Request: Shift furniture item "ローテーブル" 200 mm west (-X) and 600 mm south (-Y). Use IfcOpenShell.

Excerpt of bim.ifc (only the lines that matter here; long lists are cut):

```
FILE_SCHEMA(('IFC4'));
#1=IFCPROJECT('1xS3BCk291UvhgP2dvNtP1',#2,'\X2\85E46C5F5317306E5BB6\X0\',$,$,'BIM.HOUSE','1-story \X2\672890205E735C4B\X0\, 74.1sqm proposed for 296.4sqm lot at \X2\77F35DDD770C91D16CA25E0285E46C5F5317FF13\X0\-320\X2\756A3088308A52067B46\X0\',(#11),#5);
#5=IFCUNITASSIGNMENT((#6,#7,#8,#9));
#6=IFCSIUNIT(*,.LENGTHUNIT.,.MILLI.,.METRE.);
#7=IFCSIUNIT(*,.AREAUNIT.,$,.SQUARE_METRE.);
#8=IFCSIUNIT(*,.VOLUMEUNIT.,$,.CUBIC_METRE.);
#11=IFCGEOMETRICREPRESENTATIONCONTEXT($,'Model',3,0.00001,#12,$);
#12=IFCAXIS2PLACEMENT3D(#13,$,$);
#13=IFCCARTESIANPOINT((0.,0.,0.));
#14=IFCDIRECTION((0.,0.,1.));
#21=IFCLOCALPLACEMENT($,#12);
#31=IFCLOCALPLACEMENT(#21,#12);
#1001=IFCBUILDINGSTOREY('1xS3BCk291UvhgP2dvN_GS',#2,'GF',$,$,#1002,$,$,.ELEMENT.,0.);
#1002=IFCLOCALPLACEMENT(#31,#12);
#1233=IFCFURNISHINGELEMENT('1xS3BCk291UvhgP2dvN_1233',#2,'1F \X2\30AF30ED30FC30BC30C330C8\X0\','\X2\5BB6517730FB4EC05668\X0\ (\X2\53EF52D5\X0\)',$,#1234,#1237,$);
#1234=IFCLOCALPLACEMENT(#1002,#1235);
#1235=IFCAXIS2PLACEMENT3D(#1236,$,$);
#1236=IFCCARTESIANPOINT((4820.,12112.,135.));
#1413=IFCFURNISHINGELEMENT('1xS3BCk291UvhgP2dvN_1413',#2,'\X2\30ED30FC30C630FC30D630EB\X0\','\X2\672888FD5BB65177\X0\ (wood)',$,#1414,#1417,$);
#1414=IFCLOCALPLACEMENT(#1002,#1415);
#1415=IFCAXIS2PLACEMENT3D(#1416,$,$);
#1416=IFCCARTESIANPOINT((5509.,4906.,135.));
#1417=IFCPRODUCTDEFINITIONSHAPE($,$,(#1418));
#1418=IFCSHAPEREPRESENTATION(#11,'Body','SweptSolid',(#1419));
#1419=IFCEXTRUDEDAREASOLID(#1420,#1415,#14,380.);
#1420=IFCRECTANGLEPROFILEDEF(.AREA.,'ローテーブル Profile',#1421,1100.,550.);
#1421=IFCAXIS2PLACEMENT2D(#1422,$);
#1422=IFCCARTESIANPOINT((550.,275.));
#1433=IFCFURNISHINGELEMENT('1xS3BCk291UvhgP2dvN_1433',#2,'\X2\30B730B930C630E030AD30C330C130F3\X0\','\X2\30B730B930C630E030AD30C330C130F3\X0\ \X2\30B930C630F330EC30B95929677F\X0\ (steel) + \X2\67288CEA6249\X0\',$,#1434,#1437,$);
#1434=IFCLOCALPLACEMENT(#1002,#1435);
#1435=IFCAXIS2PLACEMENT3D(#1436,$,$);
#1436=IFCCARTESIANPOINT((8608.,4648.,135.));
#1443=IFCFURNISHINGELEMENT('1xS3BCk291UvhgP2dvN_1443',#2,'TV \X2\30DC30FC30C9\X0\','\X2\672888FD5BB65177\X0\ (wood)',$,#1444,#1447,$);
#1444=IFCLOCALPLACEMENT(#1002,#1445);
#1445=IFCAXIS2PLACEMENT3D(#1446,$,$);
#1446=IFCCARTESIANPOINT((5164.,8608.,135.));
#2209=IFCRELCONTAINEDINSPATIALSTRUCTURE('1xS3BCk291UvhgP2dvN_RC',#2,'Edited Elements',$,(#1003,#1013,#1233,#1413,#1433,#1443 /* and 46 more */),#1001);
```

```python
import ifcopenshell
import ifcopenshell.api.geometry
import ifcopenshell.util.placement
import ifcopenshell.util.unit

model = ifcopenshell.open("bim.ifc")
unit_scale = ifcopenshell.util.unit.calculate_unit_scale(model)

item = model.by_guid("1xS3BCk291UvhgP2dvN_1413")
matrix = ifcopenshell.util.placement.get_local_placement(item.ObjectPlacement)
matrix[0, 3] -= 0.2 / unit_scale
matrix[1, 3] -= 0.6 / unit_scale
ifcopenshell.api.geometry.edit_object_placement(model, product=item, matrix=matrix, is_si=False)

print(ifcopenshell.util.placement.get_local_placement(item.ObjectPlacement).round(3) + 0.0)

model.write("bim_rev.ifc")
```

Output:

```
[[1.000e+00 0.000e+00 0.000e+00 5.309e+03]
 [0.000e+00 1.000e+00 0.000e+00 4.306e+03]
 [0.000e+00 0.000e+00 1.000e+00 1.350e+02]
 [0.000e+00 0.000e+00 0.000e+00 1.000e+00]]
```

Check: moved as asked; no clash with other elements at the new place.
